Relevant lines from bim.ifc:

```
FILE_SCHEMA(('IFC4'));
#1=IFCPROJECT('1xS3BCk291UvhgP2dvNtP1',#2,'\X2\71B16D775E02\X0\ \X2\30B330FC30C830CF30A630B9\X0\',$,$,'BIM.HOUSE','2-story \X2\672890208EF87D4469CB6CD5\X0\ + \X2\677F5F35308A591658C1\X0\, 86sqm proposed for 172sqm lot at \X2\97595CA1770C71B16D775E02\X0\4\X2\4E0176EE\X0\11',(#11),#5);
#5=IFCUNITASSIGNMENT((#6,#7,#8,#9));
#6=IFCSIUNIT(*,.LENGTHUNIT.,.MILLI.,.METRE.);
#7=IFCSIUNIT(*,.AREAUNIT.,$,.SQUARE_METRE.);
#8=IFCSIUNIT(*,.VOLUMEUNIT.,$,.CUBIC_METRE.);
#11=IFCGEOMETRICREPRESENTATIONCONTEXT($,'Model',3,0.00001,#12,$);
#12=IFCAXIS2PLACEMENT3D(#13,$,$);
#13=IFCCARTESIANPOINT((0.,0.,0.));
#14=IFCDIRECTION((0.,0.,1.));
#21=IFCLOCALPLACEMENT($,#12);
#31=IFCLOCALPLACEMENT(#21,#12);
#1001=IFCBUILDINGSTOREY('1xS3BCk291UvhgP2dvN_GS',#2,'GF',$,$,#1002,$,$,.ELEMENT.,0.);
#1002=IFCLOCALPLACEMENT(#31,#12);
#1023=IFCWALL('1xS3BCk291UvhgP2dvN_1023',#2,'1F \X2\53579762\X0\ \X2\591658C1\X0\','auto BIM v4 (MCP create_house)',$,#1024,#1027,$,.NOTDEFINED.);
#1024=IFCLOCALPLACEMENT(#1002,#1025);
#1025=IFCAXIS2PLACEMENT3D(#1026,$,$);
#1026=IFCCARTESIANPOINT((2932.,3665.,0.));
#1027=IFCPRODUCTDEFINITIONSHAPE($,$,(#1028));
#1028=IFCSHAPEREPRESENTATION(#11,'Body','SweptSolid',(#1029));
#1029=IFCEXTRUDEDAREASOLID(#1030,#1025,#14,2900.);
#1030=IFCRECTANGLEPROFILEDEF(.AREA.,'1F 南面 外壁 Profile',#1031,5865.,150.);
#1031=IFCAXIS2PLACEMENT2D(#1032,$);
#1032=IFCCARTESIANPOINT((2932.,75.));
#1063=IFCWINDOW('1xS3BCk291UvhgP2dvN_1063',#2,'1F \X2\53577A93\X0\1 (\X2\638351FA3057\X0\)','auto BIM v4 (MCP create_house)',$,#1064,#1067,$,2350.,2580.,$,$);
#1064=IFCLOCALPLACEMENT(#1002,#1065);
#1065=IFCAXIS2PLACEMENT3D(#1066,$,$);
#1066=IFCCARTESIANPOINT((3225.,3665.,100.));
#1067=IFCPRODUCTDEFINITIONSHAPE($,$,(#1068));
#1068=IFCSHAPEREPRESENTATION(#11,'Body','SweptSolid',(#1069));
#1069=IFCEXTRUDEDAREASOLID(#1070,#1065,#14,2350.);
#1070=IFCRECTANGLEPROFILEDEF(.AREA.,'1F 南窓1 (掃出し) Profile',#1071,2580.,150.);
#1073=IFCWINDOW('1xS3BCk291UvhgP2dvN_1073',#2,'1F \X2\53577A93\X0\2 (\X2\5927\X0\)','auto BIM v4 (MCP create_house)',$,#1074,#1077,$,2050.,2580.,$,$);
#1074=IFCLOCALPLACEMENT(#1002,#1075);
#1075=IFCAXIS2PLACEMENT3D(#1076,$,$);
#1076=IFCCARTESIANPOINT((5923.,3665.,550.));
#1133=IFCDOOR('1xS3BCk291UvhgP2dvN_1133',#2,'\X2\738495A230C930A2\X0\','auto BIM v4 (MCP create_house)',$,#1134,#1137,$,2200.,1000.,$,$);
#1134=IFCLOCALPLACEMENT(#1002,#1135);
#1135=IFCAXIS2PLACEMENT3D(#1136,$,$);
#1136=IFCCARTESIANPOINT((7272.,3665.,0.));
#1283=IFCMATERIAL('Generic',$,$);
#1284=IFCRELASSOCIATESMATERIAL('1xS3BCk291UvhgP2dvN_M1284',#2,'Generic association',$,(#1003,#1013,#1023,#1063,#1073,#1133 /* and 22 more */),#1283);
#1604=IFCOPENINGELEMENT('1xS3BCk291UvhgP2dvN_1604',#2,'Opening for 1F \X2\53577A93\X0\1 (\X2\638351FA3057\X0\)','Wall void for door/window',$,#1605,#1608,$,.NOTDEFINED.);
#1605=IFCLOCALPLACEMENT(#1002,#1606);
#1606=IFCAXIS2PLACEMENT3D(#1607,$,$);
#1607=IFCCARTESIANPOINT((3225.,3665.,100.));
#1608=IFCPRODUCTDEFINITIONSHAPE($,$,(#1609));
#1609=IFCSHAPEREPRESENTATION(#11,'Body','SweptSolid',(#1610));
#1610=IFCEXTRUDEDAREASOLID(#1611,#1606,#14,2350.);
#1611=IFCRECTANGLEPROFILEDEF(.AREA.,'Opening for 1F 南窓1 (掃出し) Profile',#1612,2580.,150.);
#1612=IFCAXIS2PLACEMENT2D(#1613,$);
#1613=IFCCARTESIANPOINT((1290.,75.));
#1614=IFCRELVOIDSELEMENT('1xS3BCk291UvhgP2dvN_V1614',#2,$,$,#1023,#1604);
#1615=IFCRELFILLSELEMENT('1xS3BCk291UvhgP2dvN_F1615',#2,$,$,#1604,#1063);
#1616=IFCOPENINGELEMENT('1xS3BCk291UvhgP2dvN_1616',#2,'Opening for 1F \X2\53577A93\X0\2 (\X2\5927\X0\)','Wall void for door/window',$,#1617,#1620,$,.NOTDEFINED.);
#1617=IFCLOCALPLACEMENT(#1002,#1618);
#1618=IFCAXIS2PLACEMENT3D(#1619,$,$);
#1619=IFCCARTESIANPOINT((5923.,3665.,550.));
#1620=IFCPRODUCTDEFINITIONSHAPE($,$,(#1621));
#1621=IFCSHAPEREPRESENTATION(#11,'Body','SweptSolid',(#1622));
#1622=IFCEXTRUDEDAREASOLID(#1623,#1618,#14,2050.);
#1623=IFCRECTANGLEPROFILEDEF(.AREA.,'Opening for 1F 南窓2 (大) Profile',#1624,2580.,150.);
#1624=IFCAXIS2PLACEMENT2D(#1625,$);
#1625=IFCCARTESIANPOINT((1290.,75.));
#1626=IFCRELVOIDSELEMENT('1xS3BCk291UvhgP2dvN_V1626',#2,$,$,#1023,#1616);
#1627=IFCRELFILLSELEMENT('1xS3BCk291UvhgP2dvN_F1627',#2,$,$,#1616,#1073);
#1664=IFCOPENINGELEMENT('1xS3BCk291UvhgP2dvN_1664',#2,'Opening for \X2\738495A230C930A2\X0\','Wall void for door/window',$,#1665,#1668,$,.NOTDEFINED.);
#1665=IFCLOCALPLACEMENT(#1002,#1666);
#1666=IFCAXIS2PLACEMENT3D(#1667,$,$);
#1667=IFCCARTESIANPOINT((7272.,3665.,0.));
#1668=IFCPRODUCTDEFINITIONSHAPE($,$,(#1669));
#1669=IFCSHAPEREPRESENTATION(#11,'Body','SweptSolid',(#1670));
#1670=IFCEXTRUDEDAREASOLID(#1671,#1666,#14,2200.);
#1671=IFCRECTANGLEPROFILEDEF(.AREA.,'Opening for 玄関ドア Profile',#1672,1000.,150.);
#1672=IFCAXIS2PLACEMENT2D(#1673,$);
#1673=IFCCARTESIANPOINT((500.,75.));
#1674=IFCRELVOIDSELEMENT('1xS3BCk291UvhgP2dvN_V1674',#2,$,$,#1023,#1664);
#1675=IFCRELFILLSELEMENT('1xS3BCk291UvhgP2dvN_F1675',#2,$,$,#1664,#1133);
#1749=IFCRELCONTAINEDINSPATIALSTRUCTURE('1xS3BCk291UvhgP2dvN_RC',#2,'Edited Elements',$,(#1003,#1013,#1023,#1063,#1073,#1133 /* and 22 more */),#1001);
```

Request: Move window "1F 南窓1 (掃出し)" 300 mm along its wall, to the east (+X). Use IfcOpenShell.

```python
import ifcopenshell
import ifcopenshell.api.geometry
import ifcopenshell.util.placement
import ifcopenshell.util.unit

model = ifcopenshell.open("bim.ifc")
unit_scale = ifcopenshell.util.unit.calculate_unit_scale(model)

window = model.by_id(1063)
opening = window.FillsVoids[0].RelatingOpeningElement
wall = opening.VoidsElements[0].RelatingBuildingElement

wall_matrix = ifcopenshell.util.placement.get_local_placement(wall.ObjectPlacement)
shift = wall_matrix[:3, 0] * 0.3 / unit_scale
before = ifcopenshell.util.placement.get_local_placement(window.ObjectPlacement)[:3, 3].copy()

# The window is not placed relative to its opening, so move both.
for product in (opening, window):
    matrix = ifcopenshell.util.placement.get_local_placement(product.ObjectPlacement)
    matrix[:3, 3] += shift
    ifcopenshell.api.geometry.edit_object_placement(model, product=product, matrix=matrix, is_si=False)

after = ifcopenshell.util.placement.get_local_placement(window.ObjectPlacement)[:3, 3]
print("window moved by", (after - before).round(3) + 0.0)

model.write("bim_updated.ifc")
```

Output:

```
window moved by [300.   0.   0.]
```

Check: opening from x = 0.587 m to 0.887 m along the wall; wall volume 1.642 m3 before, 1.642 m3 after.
